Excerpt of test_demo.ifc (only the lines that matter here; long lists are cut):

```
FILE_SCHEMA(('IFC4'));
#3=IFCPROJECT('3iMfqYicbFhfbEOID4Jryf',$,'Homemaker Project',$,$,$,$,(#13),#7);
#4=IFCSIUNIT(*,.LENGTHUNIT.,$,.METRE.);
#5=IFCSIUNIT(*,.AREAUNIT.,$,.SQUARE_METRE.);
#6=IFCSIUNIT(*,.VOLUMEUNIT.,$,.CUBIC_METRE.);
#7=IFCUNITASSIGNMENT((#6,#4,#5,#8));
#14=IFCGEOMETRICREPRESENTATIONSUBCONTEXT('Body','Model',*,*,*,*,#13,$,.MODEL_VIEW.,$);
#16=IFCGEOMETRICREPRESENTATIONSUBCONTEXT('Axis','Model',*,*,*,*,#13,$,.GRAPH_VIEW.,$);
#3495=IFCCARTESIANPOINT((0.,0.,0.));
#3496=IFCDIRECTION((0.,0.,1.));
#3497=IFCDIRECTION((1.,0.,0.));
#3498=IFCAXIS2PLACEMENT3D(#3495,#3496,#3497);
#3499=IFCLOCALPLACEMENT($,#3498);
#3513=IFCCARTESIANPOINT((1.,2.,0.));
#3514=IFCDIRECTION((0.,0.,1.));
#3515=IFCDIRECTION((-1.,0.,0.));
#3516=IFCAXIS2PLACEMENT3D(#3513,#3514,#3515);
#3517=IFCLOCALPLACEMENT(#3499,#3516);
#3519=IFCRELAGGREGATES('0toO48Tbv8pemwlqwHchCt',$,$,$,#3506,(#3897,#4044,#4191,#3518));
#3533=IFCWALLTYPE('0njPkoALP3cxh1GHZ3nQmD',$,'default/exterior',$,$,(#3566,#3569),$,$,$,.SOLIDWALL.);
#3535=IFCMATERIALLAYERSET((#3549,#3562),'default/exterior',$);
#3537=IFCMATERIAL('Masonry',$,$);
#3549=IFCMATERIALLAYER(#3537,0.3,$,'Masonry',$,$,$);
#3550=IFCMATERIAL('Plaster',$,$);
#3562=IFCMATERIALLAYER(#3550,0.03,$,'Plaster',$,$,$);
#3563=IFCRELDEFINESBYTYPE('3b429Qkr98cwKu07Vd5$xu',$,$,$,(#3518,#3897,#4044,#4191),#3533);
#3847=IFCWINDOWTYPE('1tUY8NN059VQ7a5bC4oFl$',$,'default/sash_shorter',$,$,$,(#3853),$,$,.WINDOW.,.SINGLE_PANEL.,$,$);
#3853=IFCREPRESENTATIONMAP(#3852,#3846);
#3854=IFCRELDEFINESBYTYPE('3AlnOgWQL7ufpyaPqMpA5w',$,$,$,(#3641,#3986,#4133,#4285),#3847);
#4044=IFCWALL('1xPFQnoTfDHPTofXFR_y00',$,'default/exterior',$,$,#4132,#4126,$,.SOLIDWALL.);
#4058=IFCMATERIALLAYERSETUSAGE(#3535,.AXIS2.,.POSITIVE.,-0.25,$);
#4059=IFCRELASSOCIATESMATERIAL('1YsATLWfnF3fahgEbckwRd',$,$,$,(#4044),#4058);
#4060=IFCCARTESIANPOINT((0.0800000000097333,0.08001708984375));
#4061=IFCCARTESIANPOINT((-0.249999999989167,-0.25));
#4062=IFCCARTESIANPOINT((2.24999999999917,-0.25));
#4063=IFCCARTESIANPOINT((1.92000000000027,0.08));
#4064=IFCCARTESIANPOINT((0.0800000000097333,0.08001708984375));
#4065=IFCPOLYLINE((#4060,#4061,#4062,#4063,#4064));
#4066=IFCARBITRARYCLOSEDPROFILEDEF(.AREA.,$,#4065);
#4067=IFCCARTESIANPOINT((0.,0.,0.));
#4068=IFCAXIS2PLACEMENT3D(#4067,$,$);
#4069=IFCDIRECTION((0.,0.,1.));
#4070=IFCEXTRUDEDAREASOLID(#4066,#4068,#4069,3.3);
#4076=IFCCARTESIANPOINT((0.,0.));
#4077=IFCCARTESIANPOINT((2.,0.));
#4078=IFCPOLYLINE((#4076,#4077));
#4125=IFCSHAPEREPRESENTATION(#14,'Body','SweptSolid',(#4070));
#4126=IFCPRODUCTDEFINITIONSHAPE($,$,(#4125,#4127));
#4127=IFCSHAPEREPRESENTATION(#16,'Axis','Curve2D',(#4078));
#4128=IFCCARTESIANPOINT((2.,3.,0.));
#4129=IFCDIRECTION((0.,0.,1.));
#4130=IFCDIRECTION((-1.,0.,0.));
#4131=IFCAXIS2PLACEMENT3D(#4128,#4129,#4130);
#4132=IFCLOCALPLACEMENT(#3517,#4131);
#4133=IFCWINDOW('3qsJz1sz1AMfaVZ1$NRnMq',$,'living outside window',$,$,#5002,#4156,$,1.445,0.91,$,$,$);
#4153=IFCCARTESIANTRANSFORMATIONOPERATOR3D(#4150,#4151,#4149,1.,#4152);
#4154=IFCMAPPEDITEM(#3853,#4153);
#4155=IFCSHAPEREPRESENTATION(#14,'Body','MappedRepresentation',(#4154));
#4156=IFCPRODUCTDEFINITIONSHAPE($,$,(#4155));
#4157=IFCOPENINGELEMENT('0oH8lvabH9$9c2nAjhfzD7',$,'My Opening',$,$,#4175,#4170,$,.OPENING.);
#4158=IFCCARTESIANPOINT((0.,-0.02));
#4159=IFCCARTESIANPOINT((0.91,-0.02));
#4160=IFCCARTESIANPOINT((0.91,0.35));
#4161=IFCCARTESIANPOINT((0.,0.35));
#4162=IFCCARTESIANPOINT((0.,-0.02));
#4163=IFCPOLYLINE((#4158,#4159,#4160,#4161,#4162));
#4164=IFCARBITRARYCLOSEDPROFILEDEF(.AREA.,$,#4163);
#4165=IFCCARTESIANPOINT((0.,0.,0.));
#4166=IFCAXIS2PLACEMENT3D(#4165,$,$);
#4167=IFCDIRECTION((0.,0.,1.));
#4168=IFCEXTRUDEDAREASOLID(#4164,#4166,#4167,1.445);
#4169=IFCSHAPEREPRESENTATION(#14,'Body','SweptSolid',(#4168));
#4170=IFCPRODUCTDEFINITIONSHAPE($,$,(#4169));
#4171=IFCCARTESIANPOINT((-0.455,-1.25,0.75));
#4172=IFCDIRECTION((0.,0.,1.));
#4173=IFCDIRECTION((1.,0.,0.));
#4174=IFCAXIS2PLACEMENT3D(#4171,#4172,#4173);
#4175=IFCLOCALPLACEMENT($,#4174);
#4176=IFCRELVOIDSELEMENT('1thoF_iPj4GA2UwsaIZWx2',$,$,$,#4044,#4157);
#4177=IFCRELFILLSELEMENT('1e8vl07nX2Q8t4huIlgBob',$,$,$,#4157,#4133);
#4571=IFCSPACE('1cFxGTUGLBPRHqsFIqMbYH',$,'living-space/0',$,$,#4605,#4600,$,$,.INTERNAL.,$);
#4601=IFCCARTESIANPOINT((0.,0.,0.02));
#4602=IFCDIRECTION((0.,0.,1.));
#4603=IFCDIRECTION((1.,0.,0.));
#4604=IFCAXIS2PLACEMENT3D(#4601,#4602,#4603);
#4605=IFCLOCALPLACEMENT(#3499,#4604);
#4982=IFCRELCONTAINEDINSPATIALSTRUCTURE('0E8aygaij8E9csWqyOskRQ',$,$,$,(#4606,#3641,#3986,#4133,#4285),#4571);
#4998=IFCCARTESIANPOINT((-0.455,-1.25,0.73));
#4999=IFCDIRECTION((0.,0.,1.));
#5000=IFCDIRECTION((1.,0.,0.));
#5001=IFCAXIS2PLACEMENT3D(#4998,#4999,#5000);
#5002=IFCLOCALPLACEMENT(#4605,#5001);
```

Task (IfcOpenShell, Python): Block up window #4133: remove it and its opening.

```python
import ifcopenshell
import ifcopenshell.api.feature
import ifcopenshell.api.root
import ifcopenshell.geom
import ifcopenshell.util.shape

model = ifcopenshell.open("test_demo.ifc")
settings = ifcopenshell.geom.settings()


def volume(element):
    """Net volume in cubic metres, openings subtracted."""
    shape = ifcopenshell.geom.create_shape(settings, element)
    return ifcopenshell.util.shape.get_volume(shape.geometry)


window = model.by_guid("3qsJz1sz1AMfaVZ1$NRnMq")
opening = window.FillsVoids[0].RelatingOpeningElement
wall = opening.VoidsElements[0].RelatingBuildingElement
before = volume(wall)

ifcopenshell.api.root.remove_product(model, product=window)
ifcopenshell.api.feature.remove_feature(model, feature=opening)

after = volume(wall)

print(f"wall volume {before:.3f} -> {after:.3f} m3")

model.write("test_demo_edited.ifc")
```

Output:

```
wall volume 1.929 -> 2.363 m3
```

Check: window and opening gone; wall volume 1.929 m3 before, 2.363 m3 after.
